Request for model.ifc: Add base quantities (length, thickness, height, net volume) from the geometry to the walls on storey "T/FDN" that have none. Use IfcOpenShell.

First a look at what the model holds.

```python
import ifcopenshell
import ifcopenshell.util.element
import ifcopenshell.util.unit

model = ifcopenshell.open("model.ifc")
print(model.schema)
for unit_type in ("LENGTHUNIT", "AREAUNIT", "VOLUMEUNIT"):
    print(unit_type, ifcopenshell.util.unit.calculate_unit_scale(model, unit_type))
storey = next(s for s in model.by_type("IfcBuildingStorey") if s.Name == "T/FDN")
walls = [e for e in ifcopenshell.util.element.get_decomposition(storey) if e.is_a("IfcWall")]
for e in sorted(walls, key=lambda e: e.id()):
    print(e.id(), e.is_a(), e.Name, list(ifcopenshell.util.element.get_psets(e, qtos_only=True)), sep=" | ")
```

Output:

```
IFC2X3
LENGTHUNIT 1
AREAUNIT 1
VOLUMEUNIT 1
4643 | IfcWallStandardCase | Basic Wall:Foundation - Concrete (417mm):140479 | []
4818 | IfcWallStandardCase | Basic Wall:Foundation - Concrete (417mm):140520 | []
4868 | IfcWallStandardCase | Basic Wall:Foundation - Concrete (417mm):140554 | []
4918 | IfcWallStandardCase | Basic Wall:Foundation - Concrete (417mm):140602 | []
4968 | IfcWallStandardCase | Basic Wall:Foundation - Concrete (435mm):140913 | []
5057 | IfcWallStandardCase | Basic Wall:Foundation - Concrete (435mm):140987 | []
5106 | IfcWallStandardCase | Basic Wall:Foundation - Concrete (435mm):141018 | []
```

```python
import ifcopenshell
import ifcopenshell.api.pset
import ifcopenshell.geom
import ifcopenshell.util.element
import ifcopenshell.util.shape
import ifcopenshell.util.unit

model = ifcopenshell.open("model.ifc")
unit_scale = ifcopenshell.util.unit.calculate_unit_scale(model)
volume_scale = ifcopenshell.util.unit.calculate_unit_scale(model, "VOLUMEUNIT")
settings = ifcopenshell.geom.settings()

storey = next(s for s in model.by_type("IfcBuildingStorey") if s.Name == "T/FDN")
walls = [e for e in ifcopenshell.util.element.get_decomposition(storey) if e.is_a("IfcWall")]

for e in sorted(walls, key=lambda e: e.id()):
    if ifcopenshell.util.element.get_psets(e, qtos_only=True, should_inherit=False):
        continue
    # Geometry comes back in metres, in the element's own axes.
    shape = ifcopenshell.geom.create_shape(settings, e)
    values = {
        "Length": ifcopenshell.util.shape.get_x(shape.geometry) / unit_scale,
        "Width": ifcopenshell.util.shape.get_y(shape.geometry) / unit_scale,
        "Height": ifcopenshell.util.shape.get_z(shape.geometry) / unit_scale,
        "NetVolume": ifcopenshell.util.shape.get_volume(shape.geometry) / volume_scale,
    }
    qto = ifcopenshell.api.pset.add_qto(model, product=e, name="BaseQuantities")
    ifcopenshell.api.pset.edit_qto(model, qto=qto, properties=values)
    print(e.id(), {k: round(v, 3) for k, v in values.items()})

model.write("model_rev.ifc")
```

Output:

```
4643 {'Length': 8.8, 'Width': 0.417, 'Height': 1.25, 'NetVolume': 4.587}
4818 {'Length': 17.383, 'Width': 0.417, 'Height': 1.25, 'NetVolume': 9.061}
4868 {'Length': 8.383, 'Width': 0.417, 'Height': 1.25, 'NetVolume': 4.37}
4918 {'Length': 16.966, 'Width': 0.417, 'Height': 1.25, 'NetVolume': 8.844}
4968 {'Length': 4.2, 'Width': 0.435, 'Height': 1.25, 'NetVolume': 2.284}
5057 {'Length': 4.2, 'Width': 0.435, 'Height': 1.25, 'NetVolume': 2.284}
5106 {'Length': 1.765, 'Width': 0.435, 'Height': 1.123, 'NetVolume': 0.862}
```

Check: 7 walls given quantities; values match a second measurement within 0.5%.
